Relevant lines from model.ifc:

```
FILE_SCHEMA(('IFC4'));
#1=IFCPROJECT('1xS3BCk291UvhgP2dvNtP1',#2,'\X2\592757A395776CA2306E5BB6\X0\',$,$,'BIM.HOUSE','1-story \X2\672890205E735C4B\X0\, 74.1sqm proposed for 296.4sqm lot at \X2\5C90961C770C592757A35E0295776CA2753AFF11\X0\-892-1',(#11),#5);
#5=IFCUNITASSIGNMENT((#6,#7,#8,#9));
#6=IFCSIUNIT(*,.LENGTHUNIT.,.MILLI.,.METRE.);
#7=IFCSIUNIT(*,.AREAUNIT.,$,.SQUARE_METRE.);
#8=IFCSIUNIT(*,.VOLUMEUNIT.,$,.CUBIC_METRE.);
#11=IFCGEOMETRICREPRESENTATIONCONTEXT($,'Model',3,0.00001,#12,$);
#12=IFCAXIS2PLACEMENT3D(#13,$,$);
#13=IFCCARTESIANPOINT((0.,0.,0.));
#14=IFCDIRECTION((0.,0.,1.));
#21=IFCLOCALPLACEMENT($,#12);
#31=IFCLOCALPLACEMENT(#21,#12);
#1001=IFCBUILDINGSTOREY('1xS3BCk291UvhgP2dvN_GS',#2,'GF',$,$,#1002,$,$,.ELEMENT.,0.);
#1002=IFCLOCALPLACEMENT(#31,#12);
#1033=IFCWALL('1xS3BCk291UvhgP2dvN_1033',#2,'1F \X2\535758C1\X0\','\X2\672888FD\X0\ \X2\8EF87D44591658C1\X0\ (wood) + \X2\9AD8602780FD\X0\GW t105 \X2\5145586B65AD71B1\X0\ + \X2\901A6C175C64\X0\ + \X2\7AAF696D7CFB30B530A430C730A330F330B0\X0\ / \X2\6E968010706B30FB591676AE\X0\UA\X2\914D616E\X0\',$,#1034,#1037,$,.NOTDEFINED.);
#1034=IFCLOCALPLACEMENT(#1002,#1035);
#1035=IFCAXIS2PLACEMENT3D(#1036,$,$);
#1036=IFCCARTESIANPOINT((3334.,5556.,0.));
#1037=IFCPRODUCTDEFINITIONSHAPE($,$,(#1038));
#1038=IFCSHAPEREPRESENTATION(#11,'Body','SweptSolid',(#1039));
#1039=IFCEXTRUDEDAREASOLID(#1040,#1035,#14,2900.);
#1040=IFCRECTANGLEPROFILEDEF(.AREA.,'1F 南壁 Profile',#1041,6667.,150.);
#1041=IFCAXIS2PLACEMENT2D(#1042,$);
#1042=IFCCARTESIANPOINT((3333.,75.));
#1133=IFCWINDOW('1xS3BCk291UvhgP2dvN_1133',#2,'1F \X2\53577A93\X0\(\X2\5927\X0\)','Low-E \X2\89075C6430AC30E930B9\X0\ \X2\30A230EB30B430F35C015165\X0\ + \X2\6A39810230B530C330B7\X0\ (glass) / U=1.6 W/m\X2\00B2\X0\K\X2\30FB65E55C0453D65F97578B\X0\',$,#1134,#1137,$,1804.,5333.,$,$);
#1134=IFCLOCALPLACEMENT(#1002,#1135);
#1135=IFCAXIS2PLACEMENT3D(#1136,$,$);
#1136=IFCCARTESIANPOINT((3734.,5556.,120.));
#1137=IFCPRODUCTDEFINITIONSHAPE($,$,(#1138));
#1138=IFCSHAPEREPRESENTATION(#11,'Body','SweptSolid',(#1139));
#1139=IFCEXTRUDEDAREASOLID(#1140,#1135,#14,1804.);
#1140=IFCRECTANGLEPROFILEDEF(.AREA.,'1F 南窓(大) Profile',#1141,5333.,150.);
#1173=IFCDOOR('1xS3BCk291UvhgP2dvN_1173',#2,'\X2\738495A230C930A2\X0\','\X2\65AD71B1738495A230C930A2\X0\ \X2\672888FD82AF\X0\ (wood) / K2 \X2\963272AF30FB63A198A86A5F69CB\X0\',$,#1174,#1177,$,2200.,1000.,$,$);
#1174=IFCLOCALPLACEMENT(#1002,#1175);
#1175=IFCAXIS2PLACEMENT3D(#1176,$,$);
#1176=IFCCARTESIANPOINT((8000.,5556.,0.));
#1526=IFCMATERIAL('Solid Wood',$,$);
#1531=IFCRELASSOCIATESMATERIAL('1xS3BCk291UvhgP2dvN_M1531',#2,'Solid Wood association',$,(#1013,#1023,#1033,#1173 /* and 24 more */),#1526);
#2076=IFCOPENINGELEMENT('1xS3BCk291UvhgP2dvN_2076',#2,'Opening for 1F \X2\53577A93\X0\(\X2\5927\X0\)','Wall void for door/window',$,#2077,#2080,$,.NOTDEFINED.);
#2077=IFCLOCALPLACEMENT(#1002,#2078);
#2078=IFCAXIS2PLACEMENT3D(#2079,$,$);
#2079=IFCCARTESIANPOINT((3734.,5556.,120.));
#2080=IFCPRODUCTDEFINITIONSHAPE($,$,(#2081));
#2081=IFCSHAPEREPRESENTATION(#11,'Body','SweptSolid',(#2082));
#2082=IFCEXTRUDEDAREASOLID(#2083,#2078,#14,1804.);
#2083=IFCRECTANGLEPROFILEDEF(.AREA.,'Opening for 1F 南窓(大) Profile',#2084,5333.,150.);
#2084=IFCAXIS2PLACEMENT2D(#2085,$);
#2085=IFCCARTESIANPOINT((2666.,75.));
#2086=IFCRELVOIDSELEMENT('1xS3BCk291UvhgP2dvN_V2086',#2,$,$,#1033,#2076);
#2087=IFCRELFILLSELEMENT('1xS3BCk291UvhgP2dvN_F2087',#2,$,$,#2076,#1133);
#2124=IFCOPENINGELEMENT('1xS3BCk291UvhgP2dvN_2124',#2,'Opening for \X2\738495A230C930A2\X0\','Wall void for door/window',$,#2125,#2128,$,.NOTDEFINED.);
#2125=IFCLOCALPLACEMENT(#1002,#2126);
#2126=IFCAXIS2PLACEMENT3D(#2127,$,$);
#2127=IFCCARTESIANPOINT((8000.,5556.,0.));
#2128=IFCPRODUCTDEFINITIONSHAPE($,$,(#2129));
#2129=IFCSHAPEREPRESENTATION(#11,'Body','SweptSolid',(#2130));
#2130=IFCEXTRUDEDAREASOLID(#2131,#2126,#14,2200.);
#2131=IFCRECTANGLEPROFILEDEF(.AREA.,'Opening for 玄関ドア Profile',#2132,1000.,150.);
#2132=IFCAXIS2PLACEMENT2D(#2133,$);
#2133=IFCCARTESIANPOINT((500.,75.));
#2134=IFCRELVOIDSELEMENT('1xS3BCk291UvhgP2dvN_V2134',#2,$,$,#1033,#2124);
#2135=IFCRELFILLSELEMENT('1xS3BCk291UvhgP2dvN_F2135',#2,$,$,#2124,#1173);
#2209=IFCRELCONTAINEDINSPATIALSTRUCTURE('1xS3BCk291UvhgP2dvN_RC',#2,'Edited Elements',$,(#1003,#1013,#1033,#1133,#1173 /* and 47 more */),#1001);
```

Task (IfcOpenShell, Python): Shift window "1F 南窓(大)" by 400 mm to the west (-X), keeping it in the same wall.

```python
import ifcopenshell
import ifcopenshell.api.geometry
import ifcopenshell.util.placement
import ifcopenshell.util.unit

model = ifcopenshell.open("model.ifc")
unit_scale = ifcopenshell.util.unit.calculate_unit_scale(model)

window = model.by_id(1133)
opening = window.FillsVoids[0].RelatingOpeningElement
wall = opening.VoidsElements[0].RelatingBuildingElement

wall_matrix = ifcopenshell.util.placement.get_local_placement(wall.ObjectPlacement)
shift = wall_matrix[:3, 0] * -0.4 / unit_scale
before = ifcopenshell.util.placement.get_local_placement(window.ObjectPlacement)[:3, 3].copy()

# The window is not placed relative to its opening, so move both.
for product in (opening, window):
    matrix = ifcopenshell.util.placement.get_local_placement(product.ObjectPlacement)
    matrix[:3, 3] += shift
    ifcopenshell.api.geometry.edit_object_placement(model, product=product, matrix=matrix, is_si=False)

after = ifcopenshell.util.placement.get_local_placement(window.ObjectPlacement)[:3, 3]
print("window moved by", (after - before).round(3) + 0.0)

model.write("model_rev.ifc")
```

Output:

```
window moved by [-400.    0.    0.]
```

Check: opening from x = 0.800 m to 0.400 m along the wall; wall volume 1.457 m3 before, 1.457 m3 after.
